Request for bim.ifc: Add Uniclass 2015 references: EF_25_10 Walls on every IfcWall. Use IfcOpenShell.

First a look at what the model holds.

```python
import ifcopenshell

model = ifcopenshell.open("bim.ifc")
print(model.schema)
print("classifications:", [c.Name for c in model.by_type("IfcClassification")])
for ifc_class in ("IfcDoor", "IfcRoof", "IfcStair", "IfcWall", "IfcWindow"):
    print(ifc_class, len(model.by_type(ifc_class)))
```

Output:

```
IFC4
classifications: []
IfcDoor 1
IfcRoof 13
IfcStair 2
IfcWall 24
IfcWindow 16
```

```python
import ifcopenshell
import ifcopenshell.api.classification

model = ifcopenshell.open("bim.ifc")

system = ifcopenshell.api.classification.add_classification(model, classification="Uniclass 2015")

codes = {
    "IfcWall": ("EF_25_10", "Walls"),
}
for ifc_class, (code, name) in codes.items():
    products = model.by_type(ifc_class)
    ifcopenshell.api.classification.add_reference(
        model, products=products, classification=system, identification=code, name=name
    )
    print(code, len(products))

model.write("bim_edited.ifc")
```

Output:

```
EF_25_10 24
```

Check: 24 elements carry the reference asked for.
